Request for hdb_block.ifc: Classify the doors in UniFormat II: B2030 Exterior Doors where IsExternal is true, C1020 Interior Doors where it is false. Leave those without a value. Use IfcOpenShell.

First a look at what the model holds.

```python
import ifcopenshell
import ifcopenshell.util.element

model = ifcopenshell.open("hdb_block.ifc")
print(model.schema)
print("classifications:", [c.Name for c in model.by_type("IfcClassification")])
values = [ifcopenshell.util.element.get_pset(e, "Pset_DoorCommon", "IsExternal") for e in model.by_type("IfcDoor")]
for value in (True, False, None):
    print("IsExternal", value, values.count(value))
```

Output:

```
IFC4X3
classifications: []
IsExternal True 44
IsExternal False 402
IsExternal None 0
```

```python
import ifcopenshell
import ifcopenshell.api.classification
import ifcopenshell.util.element

model = ifcopenshell.open("hdb_block.ifc")

system = ifcopenshell.api.classification.add_classification(model, classification="UniFormat II")

doors = model.by_type("IfcDoor")
external = {e: ifcopenshell.util.element.get_pset(e, "Pset_DoorCommon", "IsExternal") for e in doors}
for flag, code, name in ((True, "B2030", "Exterior Doors"), (False, "C1020", "Interior Doors")):
    products = [e for e in doors if external[e] is flag]
    ifcopenshell.api.classification.add_reference(
        model, products=products, classification=system, identification=code, name=name
    )
    print(code, len(products))

model.write("hdb_block_v2.ifc")
```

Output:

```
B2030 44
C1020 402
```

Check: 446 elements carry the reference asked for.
